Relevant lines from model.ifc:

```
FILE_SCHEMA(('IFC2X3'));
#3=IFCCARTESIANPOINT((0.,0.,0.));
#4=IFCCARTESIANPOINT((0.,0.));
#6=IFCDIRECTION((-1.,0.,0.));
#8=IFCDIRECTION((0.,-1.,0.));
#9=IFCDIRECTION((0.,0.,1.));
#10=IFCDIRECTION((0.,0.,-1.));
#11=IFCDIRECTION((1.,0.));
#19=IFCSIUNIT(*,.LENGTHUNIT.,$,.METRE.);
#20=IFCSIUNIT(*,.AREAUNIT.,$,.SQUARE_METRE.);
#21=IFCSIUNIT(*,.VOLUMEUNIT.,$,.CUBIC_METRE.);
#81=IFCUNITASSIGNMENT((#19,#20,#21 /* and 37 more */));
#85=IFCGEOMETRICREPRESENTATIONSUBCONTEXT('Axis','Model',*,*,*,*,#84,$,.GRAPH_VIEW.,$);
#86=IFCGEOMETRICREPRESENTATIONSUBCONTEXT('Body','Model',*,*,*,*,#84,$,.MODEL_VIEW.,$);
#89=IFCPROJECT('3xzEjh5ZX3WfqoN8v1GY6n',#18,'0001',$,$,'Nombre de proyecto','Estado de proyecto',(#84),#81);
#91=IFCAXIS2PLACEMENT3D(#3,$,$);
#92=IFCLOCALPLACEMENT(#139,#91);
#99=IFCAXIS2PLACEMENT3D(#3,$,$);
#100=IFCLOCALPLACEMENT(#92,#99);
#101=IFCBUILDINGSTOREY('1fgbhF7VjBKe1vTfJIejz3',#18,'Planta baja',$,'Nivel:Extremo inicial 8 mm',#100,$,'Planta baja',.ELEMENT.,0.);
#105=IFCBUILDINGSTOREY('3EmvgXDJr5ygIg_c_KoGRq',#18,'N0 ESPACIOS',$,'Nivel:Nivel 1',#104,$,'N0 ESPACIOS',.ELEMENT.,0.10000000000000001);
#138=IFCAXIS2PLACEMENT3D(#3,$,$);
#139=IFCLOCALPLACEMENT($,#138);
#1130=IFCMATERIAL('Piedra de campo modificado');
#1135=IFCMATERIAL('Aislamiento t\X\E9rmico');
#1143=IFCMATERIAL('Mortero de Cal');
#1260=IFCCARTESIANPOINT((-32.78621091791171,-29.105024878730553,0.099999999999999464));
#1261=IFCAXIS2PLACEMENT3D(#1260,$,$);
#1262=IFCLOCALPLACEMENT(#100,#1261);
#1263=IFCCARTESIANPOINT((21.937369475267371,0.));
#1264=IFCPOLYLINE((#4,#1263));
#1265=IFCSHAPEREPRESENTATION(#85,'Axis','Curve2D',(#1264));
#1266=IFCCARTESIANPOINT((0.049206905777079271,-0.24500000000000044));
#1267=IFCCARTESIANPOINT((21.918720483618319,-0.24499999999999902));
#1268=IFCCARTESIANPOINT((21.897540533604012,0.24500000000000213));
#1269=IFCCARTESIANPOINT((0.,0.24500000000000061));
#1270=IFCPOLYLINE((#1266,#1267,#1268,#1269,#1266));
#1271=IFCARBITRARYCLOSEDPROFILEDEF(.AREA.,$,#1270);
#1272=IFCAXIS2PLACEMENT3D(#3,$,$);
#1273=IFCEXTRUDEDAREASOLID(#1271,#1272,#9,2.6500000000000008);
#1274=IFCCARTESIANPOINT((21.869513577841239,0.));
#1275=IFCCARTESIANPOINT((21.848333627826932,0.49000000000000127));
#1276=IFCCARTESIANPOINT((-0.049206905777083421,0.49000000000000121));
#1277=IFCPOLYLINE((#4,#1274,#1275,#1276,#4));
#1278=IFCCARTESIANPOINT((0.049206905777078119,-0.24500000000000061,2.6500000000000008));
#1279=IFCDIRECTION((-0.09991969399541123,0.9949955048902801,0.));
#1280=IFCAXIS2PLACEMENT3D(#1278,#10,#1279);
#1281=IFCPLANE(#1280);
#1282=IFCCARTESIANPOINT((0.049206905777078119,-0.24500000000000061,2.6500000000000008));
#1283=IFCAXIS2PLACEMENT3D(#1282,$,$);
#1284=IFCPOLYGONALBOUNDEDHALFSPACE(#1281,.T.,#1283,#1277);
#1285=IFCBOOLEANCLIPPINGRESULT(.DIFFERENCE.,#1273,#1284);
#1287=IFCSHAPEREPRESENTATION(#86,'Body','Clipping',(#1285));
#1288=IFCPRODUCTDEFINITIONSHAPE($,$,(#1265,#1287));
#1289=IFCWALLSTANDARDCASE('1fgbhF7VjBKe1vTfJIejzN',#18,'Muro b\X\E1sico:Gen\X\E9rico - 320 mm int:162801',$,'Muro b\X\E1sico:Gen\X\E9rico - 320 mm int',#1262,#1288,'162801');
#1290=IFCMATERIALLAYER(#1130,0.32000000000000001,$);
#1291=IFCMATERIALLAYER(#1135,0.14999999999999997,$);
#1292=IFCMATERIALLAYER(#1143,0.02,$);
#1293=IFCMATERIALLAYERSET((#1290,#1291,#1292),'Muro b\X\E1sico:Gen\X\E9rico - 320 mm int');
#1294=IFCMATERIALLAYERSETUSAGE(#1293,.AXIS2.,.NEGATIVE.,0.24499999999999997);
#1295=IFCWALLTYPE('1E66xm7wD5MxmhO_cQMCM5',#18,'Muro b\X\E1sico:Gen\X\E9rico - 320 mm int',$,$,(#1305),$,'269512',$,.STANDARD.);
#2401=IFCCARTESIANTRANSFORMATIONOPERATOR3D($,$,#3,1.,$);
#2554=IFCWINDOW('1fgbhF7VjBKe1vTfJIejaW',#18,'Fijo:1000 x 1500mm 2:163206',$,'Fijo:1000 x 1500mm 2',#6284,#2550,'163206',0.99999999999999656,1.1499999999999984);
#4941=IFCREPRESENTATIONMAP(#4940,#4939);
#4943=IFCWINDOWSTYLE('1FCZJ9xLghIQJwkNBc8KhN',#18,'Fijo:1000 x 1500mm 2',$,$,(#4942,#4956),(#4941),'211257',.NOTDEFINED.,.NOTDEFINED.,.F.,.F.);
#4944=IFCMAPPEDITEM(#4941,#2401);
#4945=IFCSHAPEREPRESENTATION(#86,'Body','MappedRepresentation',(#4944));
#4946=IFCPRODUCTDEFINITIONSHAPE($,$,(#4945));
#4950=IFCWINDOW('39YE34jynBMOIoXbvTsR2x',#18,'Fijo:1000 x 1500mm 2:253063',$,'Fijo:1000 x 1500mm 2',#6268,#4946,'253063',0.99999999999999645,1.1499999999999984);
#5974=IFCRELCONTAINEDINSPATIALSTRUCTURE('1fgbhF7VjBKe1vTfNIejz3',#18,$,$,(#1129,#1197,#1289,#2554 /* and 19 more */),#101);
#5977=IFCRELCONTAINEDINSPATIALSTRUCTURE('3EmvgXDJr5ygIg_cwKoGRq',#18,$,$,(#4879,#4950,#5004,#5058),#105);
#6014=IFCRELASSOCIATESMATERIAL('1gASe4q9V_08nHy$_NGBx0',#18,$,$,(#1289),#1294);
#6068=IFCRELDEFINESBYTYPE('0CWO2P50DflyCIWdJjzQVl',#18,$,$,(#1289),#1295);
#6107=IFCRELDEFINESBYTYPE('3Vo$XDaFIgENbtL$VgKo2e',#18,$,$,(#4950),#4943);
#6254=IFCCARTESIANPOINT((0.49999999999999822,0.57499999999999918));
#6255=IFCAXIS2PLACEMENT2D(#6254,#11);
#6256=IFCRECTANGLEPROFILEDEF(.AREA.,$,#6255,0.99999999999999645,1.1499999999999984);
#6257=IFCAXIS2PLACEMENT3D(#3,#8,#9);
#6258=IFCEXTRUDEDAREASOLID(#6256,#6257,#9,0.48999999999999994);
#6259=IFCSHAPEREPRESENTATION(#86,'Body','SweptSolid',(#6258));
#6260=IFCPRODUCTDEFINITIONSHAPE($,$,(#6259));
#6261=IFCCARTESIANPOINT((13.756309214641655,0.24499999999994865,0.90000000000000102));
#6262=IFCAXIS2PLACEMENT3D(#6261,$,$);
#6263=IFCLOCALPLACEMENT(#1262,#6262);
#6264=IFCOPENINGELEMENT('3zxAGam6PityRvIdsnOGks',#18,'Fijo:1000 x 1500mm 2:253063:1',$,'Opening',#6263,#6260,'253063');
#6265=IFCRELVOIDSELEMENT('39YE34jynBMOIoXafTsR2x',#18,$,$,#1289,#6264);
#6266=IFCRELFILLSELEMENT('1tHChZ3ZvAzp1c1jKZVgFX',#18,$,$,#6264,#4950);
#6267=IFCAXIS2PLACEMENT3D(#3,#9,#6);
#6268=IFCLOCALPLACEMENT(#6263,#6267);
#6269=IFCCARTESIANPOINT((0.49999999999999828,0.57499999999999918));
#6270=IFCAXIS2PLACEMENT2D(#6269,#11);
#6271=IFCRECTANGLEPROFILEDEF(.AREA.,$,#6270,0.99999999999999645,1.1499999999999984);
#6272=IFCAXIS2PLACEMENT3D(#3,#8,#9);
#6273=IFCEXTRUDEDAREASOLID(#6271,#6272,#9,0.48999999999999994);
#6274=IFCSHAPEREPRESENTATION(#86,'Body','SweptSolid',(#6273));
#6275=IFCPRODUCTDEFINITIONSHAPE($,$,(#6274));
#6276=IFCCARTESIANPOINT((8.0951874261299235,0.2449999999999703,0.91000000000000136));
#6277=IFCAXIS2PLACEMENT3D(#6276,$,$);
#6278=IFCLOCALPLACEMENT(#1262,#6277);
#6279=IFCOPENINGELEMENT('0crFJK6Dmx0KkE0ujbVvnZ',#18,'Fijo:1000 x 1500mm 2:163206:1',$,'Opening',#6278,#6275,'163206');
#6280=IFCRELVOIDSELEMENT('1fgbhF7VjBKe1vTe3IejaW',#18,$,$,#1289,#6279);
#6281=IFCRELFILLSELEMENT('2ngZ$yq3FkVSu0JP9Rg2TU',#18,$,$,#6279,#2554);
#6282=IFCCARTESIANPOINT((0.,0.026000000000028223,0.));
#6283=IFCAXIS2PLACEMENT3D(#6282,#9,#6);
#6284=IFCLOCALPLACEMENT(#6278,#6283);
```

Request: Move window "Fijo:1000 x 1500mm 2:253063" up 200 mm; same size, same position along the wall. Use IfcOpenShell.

```python
import numpy as np
import ifcopenshell
import ifcopenshell.api.geometry
import ifcopenshell.util.placement
import ifcopenshell.util.unit

model = ifcopenshell.open("model.ifc")
unit_scale = ifcopenshell.util.unit.calculate_unit_scale(model)

window = model.by_id(4950)
opening = window.FillsVoids[0].RelatingOpeningElement
dz = 0.2 / unit_scale

shift = np.array([0.0, 0.0, dz])
# The window is placed relative to its opening, so it follows when the opening moves.
matrix = ifcopenshell.util.placement.get_local_placement(opening.ObjectPlacement)
matrix[:3, 3] += shift
ifcopenshell.api.geometry.edit_object_placement(
    model, product=opening, matrix=matrix, is_si=False, should_transform_children=True
)

print(f"moved by {dz * unit_scale:+.3f} m")

model.write("model_edited.ifc")
```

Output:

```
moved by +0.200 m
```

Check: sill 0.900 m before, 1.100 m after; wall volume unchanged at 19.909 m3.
